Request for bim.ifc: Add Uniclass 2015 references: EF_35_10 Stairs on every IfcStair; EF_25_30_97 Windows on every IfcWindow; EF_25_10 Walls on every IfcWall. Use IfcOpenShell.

First a look at what the model holds.

```python
import ifcopenshell

model = ifcopenshell.open("bim.ifc")
print(model.schema)
print("classifications:", [c.Name for c in model.by_type("IfcClassification")])
for ifc_class in ("IfcDoor", "IfcRoof", "IfcStair", "IfcWall", "IfcWindow"):
    print(ifc_class, len(model.by_type(ifc_class)))
```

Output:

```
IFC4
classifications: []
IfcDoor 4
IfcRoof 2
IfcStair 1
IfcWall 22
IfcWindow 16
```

```python
import ifcopenshell
import ifcopenshell.api.classification

model = ifcopenshell.open("bim.ifc")

system = ifcopenshell.api.classification.add_classification(model, classification="Uniclass 2015")

codes = {
    "IfcStair": ("EF_35_10", "Stairs"),
    "IfcWindow": ("EF_25_30_97", "Windows"),
    "IfcWall": ("EF_25_10", "Walls"),
}
for ifc_class, (code, name) in codes.items():
    products = model.by_type(ifc_class)
    ifcopenshell.api.classification.add_reference(
        model, products=products, classification=system, identification=code, name=name
    )
    print(code, len(products))

model.write("bim_rev.ifc")
```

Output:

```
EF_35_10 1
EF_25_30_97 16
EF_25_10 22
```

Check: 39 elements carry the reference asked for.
